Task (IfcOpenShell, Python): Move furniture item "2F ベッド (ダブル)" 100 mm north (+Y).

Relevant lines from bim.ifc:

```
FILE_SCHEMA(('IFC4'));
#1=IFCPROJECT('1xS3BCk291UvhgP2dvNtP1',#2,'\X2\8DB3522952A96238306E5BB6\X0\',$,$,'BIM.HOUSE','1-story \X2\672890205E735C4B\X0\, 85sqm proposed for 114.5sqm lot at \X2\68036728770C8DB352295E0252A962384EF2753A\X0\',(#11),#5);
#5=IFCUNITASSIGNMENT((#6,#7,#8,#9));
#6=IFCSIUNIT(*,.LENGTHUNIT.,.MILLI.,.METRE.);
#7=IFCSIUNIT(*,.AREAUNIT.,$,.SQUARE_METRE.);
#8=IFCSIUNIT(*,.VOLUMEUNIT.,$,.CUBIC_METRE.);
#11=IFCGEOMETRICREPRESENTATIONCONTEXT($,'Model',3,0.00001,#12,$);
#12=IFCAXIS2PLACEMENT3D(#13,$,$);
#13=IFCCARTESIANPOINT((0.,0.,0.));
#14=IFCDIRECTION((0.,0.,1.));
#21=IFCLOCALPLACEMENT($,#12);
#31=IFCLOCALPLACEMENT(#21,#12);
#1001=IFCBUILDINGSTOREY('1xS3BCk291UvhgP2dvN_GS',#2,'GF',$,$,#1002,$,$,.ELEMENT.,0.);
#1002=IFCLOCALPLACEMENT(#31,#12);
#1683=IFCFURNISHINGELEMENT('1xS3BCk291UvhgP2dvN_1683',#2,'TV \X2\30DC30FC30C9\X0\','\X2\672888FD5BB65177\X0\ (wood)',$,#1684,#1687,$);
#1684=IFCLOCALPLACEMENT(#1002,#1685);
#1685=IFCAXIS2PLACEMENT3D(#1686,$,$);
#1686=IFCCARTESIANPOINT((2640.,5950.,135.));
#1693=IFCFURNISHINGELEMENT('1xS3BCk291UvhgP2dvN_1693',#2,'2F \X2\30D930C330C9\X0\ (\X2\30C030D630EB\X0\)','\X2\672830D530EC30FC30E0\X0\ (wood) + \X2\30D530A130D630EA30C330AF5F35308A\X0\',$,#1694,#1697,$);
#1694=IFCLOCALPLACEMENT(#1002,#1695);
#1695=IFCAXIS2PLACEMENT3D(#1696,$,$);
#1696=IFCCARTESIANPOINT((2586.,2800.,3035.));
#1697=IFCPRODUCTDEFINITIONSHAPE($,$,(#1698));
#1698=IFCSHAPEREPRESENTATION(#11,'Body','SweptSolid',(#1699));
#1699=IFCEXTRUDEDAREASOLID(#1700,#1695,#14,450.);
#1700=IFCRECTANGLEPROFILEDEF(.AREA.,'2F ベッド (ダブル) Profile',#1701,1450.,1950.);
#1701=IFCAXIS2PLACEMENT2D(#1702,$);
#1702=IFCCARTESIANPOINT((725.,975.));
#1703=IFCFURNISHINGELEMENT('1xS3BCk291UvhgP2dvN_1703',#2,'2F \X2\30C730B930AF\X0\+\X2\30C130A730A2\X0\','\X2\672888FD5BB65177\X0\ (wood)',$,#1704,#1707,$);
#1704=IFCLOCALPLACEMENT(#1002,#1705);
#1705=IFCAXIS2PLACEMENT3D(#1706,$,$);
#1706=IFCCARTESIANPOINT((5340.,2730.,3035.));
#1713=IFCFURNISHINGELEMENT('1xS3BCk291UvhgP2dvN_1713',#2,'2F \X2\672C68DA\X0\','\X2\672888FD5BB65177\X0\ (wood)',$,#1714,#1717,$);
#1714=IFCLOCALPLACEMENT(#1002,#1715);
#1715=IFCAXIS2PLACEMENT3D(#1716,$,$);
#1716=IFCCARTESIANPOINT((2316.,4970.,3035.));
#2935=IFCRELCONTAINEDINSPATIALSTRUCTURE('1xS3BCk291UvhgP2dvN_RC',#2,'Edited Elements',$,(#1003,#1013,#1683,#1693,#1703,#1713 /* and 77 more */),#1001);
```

```python
import ifcopenshell
import ifcopenshell.api.geometry
import ifcopenshell.util.placement
import ifcopenshell.util.unit

model = ifcopenshell.open("bim.ifc")
unit_scale = ifcopenshell.util.unit.calculate_unit_scale(model)

item = model.by_id(1693)
matrix = ifcopenshell.util.placement.get_local_placement(item.ObjectPlacement)
matrix[1, 3] += 0.1 / unit_scale
ifcopenshell.api.geometry.edit_object_placement(model, product=item, matrix=matrix, is_si=False)

print(ifcopenshell.util.placement.get_local_placement(item.ObjectPlacement).round(3) + 0.0)

model.write("bim-out.ifc")
```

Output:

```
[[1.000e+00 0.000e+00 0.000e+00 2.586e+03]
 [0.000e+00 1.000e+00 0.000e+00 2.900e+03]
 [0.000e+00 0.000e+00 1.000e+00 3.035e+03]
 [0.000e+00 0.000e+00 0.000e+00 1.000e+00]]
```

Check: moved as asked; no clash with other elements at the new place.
